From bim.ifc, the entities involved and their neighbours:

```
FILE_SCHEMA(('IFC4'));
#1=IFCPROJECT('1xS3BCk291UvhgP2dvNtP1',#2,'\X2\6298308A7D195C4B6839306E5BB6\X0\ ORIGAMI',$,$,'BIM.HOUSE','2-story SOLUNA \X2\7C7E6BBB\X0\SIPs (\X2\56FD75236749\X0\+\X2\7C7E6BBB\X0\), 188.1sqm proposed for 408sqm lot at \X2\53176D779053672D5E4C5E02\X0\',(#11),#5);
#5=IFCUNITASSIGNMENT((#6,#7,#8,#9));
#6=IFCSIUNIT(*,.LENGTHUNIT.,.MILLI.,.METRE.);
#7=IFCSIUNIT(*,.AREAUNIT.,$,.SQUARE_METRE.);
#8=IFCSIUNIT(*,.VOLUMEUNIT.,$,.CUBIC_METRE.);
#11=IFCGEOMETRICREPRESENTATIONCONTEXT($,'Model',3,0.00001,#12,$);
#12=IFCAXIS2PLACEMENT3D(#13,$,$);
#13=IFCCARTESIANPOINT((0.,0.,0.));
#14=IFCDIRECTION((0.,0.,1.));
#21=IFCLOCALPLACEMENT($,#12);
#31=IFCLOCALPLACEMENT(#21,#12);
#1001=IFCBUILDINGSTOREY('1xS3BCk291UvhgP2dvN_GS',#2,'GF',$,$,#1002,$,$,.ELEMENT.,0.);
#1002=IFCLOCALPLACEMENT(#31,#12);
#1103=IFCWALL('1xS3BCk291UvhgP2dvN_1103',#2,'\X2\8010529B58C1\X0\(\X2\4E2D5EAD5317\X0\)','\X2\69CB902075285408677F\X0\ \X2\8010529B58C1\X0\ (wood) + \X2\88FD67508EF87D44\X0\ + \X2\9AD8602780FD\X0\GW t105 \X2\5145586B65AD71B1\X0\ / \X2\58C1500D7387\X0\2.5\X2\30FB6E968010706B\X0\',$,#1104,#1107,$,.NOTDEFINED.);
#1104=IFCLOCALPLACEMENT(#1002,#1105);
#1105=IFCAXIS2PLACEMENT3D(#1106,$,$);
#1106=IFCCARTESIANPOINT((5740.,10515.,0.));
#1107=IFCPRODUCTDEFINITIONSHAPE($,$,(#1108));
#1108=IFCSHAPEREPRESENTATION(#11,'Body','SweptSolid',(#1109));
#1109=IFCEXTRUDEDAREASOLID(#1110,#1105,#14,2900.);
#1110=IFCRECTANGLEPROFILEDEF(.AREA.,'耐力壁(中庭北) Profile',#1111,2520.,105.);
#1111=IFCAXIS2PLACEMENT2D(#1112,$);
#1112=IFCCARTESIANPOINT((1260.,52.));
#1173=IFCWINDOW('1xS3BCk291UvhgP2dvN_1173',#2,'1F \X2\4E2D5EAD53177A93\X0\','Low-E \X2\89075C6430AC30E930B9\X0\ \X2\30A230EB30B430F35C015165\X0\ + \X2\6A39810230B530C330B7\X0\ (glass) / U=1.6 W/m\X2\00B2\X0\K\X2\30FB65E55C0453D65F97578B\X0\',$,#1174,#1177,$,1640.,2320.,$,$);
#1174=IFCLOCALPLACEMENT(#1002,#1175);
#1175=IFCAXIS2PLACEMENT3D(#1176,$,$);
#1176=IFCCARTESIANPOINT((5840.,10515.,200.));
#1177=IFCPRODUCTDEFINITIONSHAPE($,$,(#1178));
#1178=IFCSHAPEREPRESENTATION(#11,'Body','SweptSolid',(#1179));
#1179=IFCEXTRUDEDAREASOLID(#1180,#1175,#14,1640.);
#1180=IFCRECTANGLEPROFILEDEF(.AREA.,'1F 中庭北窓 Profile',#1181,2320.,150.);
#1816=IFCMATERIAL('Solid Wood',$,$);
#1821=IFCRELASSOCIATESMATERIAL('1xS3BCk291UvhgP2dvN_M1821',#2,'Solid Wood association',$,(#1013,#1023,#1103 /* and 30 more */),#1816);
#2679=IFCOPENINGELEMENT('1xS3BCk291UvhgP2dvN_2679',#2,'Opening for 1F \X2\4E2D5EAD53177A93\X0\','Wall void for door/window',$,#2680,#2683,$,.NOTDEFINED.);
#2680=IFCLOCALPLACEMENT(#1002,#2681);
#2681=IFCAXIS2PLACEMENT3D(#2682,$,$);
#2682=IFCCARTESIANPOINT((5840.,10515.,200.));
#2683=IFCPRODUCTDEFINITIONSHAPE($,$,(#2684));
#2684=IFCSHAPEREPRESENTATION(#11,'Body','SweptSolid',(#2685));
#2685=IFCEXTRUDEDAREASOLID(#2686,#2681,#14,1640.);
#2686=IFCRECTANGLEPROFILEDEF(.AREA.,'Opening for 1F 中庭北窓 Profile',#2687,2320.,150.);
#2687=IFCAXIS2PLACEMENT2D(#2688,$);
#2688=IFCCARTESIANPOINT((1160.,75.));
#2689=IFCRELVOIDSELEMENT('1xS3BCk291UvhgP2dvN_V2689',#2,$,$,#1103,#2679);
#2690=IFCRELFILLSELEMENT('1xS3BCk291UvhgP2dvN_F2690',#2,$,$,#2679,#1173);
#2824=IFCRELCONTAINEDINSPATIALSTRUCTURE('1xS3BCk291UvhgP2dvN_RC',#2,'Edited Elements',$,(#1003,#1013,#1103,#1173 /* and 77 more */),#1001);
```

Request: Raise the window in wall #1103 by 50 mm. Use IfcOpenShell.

```python
import numpy as np
import ifcopenshell
import ifcopenshell.api.geometry
import ifcopenshell.util.placement
import ifcopenshell.util.unit

model = ifcopenshell.open("bim.ifc")
unit_scale = ifcopenshell.util.unit.calculate_unit_scale(model)

window = model.by_guid("1xS3BCk291UvhgP2dvN_1173")
opening = window.FillsVoids[0].RelatingOpeningElement
dz = 50.0

shift = np.array([0.0, 0.0, dz])
# The window is not placed relative to its opening, so move both.
for product in (opening, window):
    matrix = ifcopenshell.util.placement.get_local_placement(product.ObjectPlacement)
    matrix[:3, 3] += shift
    ifcopenshell.api.geometry.edit_object_placement(model, product=product, matrix=matrix, is_si=False)

print(f"moved by {dz * unit_scale:+.3f} m")

model.write("bim_rev.ifc")
```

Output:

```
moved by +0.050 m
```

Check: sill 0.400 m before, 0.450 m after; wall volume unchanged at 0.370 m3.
